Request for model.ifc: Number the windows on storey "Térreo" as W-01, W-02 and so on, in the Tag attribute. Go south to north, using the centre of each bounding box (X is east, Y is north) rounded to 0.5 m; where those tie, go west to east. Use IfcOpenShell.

First a look at what the model holds.

```python
import ifcopenshell
import ifcopenshell.util.element
import ifcopenshell.util.placement

model = ifcopenshell.open("model.ifc")
print(model.schema)
storey = next(s for s in model.by_type("IfcBuildingStorey") if s.Name == "Térreo")
windows = [e for e in ifcopenshell.util.element.get_decomposition(storey) if e.is_a("IfcWindow")]
for e in sorted(windows, key=lambda e: e.id()):
    origin = ifcopenshell.util.placement.get_local_placement(e.ObjectPlacement)[:3, 3]
    print(e.id(), e.Tag, e.Name, origin.round(2) + 0.0, sep=" | ")
```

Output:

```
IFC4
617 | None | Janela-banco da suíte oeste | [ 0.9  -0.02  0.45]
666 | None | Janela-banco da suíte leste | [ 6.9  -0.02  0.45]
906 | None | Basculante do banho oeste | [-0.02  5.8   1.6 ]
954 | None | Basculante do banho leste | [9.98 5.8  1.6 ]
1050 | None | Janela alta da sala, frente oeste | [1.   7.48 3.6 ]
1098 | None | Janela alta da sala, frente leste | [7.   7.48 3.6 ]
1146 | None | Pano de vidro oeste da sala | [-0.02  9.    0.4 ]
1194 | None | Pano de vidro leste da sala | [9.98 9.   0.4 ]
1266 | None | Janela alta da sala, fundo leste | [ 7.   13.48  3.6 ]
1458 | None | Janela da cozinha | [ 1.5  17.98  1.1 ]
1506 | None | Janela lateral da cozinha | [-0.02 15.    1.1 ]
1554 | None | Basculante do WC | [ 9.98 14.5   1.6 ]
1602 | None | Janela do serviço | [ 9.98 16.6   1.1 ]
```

```python
import ifcopenshell
import ifcopenshell.geom
import ifcopenshell.util.element
import ifcopenshell.util.shape

model = ifcopenshell.open("model.ifc")
settings = ifcopenshell.geom.settings()
settings.set("use-world-coords", True)


def centre(element):
    shape = ifcopenshell.geom.create_shape(settings, element)
    return ifcopenshell.util.shape.get_bbox_centroid(shape.geometry)


storey = next(s for s in model.by_type("IfcBuildingStorey") if s.Name == "Térreo")
windows = [e for e in ifcopenshell.util.element.get_decomposition(storey) if e.is_a("IfcWindow")]

# Insertion points can sit at a corner or the storey origin, so sort by the geometry (in metres).
centres = {e: centre(e) for e in windows}
windows.sort(key=lambda e: (round(centres[e][1] / 0.5), centres[e][0]))

for i, e in enumerate(windows, start=1):
    number = f"W-{i:02d}"
    e.Tag = number
    print(e.id(), number)

model.write("model-out.ifc")
```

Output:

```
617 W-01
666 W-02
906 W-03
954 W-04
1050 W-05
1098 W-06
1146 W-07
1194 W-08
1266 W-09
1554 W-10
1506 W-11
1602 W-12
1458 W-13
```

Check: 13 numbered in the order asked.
